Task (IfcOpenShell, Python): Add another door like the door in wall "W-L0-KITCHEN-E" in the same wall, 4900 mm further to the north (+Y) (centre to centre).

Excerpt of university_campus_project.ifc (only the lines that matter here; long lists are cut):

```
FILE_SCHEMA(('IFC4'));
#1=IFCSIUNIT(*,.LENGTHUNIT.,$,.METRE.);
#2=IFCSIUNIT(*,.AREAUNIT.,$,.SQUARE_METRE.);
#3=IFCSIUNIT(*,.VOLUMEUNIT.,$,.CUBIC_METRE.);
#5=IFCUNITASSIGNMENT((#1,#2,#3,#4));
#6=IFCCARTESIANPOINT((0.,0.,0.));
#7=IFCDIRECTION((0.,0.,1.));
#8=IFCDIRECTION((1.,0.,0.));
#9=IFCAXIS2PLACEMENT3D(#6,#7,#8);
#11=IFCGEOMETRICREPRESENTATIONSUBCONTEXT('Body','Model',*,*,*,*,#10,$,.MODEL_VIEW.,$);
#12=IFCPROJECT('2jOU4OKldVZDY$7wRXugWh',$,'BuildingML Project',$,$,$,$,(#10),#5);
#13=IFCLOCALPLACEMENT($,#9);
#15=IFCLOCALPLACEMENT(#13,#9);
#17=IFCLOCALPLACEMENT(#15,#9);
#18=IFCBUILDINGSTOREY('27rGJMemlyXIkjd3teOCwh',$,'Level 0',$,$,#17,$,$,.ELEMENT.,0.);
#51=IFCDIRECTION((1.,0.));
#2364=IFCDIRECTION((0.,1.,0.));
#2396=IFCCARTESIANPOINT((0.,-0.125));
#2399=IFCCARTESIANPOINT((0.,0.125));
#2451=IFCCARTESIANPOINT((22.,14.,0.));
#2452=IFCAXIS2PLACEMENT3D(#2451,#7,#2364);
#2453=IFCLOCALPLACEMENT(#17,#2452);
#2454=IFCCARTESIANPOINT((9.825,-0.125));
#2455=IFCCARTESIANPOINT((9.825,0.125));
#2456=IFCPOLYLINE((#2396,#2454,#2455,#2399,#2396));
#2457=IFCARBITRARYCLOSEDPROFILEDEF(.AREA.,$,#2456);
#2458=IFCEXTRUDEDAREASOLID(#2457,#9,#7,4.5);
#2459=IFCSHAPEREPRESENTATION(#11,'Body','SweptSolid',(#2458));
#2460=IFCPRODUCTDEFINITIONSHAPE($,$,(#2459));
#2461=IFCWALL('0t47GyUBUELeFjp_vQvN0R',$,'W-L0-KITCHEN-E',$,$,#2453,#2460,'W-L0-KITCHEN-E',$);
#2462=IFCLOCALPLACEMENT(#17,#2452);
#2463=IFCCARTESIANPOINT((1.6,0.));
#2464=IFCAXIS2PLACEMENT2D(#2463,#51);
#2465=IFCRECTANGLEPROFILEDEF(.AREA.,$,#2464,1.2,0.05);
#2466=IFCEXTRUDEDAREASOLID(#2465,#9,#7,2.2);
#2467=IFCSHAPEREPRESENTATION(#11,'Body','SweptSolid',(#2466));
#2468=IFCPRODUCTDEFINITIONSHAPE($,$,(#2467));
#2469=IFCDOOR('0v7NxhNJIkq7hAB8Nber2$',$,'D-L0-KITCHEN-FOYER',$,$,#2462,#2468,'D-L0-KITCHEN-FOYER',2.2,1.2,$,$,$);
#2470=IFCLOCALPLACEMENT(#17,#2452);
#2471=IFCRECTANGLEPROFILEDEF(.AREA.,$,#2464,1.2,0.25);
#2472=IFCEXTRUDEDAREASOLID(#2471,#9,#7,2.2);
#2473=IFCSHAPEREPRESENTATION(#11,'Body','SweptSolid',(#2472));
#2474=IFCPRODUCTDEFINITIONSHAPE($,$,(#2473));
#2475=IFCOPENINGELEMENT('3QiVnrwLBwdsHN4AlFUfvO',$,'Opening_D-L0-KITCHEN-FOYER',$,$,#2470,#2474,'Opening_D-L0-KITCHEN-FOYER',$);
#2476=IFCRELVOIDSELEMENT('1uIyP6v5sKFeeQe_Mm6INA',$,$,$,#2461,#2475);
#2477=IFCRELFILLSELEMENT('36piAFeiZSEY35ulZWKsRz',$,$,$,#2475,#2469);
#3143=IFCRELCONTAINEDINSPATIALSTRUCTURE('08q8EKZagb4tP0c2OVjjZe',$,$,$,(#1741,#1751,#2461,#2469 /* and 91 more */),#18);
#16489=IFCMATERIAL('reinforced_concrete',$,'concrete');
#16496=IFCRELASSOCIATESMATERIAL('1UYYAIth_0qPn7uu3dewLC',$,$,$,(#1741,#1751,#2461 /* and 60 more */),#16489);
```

```python
import ifcopenshell
import ifcopenshell.api.feature
import ifcopenshell.api.geometry
import ifcopenshell.api.root
import ifcopenshell.geom
import ifcopenshell.util.element
import ifcopenshell.util.placement
import ifcopenshell.util.shape
import ifcopenshell.util.unit

model = ifcopenshell.open("university_campus_project.ifc")
unit_scale = ifcopenshell.util.unit.calculate_unit_scale(model)
settings = ifcopenshell.geom.settings()


def volume(element):
    """Net volume in cubic metres, openings subtracted."""
    shape = ifcopenshell.geom.create_shape(settings, element)
    return ifcopenshell.util.shape.get_volume(shape.geometry)


door = model.by_guid("0v7NxhNJIkq7hAB8Nber2$")
opening = door.FillsVoids[0].RelatingOpeningElement
wall = opening.VoidsElements[0].RelatingBuildingElement
before = volume(wall)
shift = ifcopenshell.util.placement.get_local_placement(wall.ObjectPlacement)[:3, 0] * 4.9 / unit_scale

# copy_class copies the void relationship, type, container and properties, but no geometry.
new_opening = ifcopenshell.api.root.copy_class(model, product=opening)
new_opening.Representation = ifcopenshell.util.element.copy_deep(
    model, opening.Representation, exclude=["IfcGeometricRepresentationContext", "IfcRepresentationMap"]
)
new_opening.Tag = None
new_door = ifcopenshell.api.root.copy_class(model, product=door)
new_door.Representation = ifcopenshell.util.element.copy_deep(
    model, door.Representation, exclude=["IfcGeometricRepresentationContext", "IfcRepresentationMap"]
)
new_door.Tag = None
ifcopenshell.api.feature.add_filling(model, opening=new_opening, element=new_door)

for old, new in ((opening, new_opening), (door, new_door)):
    matrix = ifcopenshell.util.placement.get_local_placement(old.ObjectPlacement)
    matrix[:3, 3] += shift
    ifcopenshell.api.geometry.edit_object_placement(model, product=new, matrix=matrix, is_si=False)

after = volume(wall)

print(f"wall volume {before:.3f} -> {after:.3f} m3")

model.write("university_campus_project_updated.ifc")
```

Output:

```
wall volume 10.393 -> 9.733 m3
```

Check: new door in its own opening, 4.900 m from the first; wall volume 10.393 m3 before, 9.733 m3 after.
